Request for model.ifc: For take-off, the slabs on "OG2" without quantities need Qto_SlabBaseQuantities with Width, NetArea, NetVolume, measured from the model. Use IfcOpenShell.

First a look at what the model holds.

```python
import ifcopenshell
import ifcopenshell.util.element
import ifcopenshell.util.unit

model = ifcopenshell.open("model.ifc")
print(model.schema)
for unit_type in ("LENGTHUNIT", "AREAUNIT", "VOLUMEUNIT"):
    print(unit_type, ifcopenshell.util.unit.calculate_unit_scale(model, unit_type))
storey = next(s for s in model.by_type("IfcBuildingStorey") if s.Name == "OG2")
slabs = [e for e in ifcopenshell.util.element.get_decomposition(storey) if e.is_a("IfcSlab")]
for e in sorted(slabs, key=lambda e: e.id()):
    print(e.id(), e.is_a(), e.Name, list(ifcopenshell.util.element.get_psets(e, qtos_only=True)), sep=" | ")
```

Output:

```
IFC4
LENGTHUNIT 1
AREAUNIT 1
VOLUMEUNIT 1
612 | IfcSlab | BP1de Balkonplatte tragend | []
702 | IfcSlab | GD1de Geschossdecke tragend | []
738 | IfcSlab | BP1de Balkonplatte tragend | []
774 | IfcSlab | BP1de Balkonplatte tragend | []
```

```python
import ifcopenshell
import ifcopenshell.api.pset
import ifcopenshell.geom
import ifcopenshell.util.element
import ifcopenshell.util.shape
import ifcopenshell.util.unit

model = ifcopenshell.open("model.ifc")
unit_scale = ifcopenshell.util.unit.calculate_unit_scale(model)
area_scale = ifcopenshell.util.unit.calculate_unit_scale(model, "AREAUNIT")
volume_scale = ifcopenshell.util.unit.calculate_unit_scale(model, "VOLUMEUNIT")
settings = ifcopenshell.geom.settings()

storey = next(s for s in model.by_type("IfcBuildingStorey") if s.Name == "OG2")
slabs = [e for e in ifcopenshell.util.element.get_decomposition(storey) if e.is_a("IfcSlab")]

for e in sorted(slabs, key=lambda e: e.id()):
    if ifcopenshell.util.element.get_psets(e, qtos_only=True, should_inherit=False):
        continue
    # Geometry comes back in metres, in the element's own axes.
    shape = ifcopenshell.geom.create_shape(settings, e)
    values = {
        "Width": ifcopenshell.util.shape.get_z(shape.geometry) / unit_scale,
        "NetArea": ifcopenshell.util.shape.get_footprint_area(shape.geometry) / area_scale,
        "NetVolume": ifcopenshell.util.shape.get_volume(shape.geometry) / volume_scale,
    }
    qto = ifcopenshell.api.pset.add_qto(model, product=e, name="Qto_SlabBaseQuantities")
    ifcopenshell.api.pset.edit_qto(model, qto=qto, properties=values)
    print(e.id(), {k: round(v, 3) for k, v in values.items()})

model.write("model_edited.ifc")
```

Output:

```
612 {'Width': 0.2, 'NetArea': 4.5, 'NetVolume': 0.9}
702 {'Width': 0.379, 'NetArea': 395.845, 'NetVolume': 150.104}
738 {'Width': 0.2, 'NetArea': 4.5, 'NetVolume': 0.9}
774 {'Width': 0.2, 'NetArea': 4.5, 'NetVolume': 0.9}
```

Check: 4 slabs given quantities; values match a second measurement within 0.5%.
